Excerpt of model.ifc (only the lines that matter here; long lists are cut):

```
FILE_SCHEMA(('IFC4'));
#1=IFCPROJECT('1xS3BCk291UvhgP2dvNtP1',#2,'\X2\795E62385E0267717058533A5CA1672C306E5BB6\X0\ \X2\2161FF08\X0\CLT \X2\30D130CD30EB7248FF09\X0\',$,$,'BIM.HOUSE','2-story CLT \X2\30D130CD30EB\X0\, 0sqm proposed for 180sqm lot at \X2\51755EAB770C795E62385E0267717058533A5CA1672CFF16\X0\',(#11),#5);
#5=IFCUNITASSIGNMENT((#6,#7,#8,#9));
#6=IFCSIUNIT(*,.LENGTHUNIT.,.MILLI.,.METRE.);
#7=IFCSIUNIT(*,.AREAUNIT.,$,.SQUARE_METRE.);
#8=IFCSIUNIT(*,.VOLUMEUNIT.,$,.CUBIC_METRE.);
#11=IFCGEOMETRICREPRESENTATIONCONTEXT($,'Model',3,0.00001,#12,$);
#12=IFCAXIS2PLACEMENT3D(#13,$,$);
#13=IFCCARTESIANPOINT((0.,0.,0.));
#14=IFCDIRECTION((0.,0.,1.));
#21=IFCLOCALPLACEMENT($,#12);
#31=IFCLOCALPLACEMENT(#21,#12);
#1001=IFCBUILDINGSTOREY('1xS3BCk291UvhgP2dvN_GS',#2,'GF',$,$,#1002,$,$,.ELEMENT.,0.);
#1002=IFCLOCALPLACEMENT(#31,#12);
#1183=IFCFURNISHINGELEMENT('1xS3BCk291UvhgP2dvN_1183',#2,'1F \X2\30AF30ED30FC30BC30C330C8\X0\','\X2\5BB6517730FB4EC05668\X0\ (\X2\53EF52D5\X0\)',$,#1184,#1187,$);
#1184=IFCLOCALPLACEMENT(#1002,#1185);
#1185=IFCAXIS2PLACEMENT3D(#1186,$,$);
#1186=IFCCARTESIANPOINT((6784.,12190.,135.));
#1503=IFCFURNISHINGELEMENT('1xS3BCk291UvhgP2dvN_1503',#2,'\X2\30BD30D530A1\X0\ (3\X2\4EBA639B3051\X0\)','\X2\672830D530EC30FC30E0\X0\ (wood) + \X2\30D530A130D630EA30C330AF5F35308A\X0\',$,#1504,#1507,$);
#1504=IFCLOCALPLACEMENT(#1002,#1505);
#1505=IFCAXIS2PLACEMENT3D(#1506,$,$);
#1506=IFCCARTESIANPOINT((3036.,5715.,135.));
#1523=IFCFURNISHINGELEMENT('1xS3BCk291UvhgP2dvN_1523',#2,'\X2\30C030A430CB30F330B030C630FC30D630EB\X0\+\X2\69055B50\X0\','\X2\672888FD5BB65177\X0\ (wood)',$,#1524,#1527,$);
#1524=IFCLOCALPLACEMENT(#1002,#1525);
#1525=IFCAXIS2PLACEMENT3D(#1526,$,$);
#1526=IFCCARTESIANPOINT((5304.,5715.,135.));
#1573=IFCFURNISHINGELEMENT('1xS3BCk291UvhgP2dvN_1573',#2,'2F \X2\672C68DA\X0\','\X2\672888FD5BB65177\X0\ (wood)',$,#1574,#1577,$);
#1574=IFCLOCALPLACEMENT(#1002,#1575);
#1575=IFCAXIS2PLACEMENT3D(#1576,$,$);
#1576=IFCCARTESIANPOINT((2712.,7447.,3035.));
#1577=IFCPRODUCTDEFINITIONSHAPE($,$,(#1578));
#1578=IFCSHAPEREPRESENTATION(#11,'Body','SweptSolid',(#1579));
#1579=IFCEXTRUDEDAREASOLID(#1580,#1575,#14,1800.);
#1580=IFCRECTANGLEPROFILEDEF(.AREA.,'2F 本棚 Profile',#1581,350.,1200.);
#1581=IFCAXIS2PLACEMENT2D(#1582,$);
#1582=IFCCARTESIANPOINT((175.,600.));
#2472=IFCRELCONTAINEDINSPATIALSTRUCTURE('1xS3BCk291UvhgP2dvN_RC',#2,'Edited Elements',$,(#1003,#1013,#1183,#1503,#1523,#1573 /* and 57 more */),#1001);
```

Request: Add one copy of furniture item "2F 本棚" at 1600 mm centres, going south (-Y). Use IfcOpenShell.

```python
import numpy as np
import ifcopenshell
import ifcopenshell.api.geometry
import ifcopenshell.api.root
import ifcopenshell.util.element
import ifcopenshell.util.placement
import ifcopenshell.util.unit

model = ifcopenshell.open("model.ifc")
unit_scale = ifcopenshell.util.unit.calculate_unit_scale(model)


def reuse_history(source, copy):
    """copy_class also copies each property set's owner history, people and application; keep the originals."""
    for rel in copy.IsDefinedBy:
        if rel.is_a("IfcRelDefinesByProperties") and (history := rel.RelatingPropertyDefinition.OwnerHistory):
            rel.RelatingPropertyDefinition.OwnerHistory = source.OwnerHistory
            ifcopenshell.util.element.remove_deep2(model, history)


source = model.by_guid("1xS3BCk291UvhgP2dvN_1573")
base = ifcopenshell.util.placement.get_local_placement(source.ObjectPlacement)
step = np.array([0.0, -1.0, 0.0]) * 1.6 / unit_scale

for i in range(1, 2):
    copy = ifcopenshell.api.root.copy_class(model, product=source)
    copy.Representation = ifcopenshell.util.element.copy_deep(
        model, source.Representation, exclude=["IfcGeometricRepresentationContext", "IfcRepresentationMap"]
    )
    reuse_history(source, copy)
    matrix = base.copy()
    matrix[:3, 3] += i * step
    print("added at", matrix[:3, 3].round(3) + 0.0)
    ifcopenshell.api.geometry.edit_object_placement(model, product=copy, matrix=matrix, is_si=False)

model.write("model_rev.ifc")
```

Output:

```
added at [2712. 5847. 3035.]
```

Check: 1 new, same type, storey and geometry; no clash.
